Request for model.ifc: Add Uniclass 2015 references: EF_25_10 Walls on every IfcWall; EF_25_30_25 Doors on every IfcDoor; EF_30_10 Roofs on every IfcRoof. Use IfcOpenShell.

First a look at what the model holds.

```python
import ifcopenshell

model = ifcopenshell.open("model.ifc")
print(model.schema)
print("classifications:", [c.Name for c in model.by_type("IfcClassification")])
for ifc_class in ("IfcDoor", "IfcRoof", "IfcStair", "IfcWall", "IfcWindow"):
    print(ifc_class, len(model.by_type(ifc_class)))
```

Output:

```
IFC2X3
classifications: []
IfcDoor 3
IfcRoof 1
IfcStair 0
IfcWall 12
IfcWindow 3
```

```python
import ifcopenshell
import ifcopenshell.api.classification

model = ifcopenshell.open("model.ifc")

# IFC2X3 requires Source and Edition and has no link from the project to the system.
system = model.create_entity("IfcClassification", Source="NBS", Edition="2015", Name="Uniclass 2015")

codes = {
    "IfcWall": ("EF_25_10", "Walls"),
    "IfcDoor": ("EF_25_30_25", "Doors"),
    "IfcRoof": ("EF_30_10", "Roofs"),
}
for ifc_class, (code, name) in codes.items():
    products = model.by_type(ifc_class)
    ifcopenshell.api.classification.add_reference(
        model, products=products, classification=system, identification=code, name=name
    )
    print(code, len(products))

model.write("model_v2.ifc")
```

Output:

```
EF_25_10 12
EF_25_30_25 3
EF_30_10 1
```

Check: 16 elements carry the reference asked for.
